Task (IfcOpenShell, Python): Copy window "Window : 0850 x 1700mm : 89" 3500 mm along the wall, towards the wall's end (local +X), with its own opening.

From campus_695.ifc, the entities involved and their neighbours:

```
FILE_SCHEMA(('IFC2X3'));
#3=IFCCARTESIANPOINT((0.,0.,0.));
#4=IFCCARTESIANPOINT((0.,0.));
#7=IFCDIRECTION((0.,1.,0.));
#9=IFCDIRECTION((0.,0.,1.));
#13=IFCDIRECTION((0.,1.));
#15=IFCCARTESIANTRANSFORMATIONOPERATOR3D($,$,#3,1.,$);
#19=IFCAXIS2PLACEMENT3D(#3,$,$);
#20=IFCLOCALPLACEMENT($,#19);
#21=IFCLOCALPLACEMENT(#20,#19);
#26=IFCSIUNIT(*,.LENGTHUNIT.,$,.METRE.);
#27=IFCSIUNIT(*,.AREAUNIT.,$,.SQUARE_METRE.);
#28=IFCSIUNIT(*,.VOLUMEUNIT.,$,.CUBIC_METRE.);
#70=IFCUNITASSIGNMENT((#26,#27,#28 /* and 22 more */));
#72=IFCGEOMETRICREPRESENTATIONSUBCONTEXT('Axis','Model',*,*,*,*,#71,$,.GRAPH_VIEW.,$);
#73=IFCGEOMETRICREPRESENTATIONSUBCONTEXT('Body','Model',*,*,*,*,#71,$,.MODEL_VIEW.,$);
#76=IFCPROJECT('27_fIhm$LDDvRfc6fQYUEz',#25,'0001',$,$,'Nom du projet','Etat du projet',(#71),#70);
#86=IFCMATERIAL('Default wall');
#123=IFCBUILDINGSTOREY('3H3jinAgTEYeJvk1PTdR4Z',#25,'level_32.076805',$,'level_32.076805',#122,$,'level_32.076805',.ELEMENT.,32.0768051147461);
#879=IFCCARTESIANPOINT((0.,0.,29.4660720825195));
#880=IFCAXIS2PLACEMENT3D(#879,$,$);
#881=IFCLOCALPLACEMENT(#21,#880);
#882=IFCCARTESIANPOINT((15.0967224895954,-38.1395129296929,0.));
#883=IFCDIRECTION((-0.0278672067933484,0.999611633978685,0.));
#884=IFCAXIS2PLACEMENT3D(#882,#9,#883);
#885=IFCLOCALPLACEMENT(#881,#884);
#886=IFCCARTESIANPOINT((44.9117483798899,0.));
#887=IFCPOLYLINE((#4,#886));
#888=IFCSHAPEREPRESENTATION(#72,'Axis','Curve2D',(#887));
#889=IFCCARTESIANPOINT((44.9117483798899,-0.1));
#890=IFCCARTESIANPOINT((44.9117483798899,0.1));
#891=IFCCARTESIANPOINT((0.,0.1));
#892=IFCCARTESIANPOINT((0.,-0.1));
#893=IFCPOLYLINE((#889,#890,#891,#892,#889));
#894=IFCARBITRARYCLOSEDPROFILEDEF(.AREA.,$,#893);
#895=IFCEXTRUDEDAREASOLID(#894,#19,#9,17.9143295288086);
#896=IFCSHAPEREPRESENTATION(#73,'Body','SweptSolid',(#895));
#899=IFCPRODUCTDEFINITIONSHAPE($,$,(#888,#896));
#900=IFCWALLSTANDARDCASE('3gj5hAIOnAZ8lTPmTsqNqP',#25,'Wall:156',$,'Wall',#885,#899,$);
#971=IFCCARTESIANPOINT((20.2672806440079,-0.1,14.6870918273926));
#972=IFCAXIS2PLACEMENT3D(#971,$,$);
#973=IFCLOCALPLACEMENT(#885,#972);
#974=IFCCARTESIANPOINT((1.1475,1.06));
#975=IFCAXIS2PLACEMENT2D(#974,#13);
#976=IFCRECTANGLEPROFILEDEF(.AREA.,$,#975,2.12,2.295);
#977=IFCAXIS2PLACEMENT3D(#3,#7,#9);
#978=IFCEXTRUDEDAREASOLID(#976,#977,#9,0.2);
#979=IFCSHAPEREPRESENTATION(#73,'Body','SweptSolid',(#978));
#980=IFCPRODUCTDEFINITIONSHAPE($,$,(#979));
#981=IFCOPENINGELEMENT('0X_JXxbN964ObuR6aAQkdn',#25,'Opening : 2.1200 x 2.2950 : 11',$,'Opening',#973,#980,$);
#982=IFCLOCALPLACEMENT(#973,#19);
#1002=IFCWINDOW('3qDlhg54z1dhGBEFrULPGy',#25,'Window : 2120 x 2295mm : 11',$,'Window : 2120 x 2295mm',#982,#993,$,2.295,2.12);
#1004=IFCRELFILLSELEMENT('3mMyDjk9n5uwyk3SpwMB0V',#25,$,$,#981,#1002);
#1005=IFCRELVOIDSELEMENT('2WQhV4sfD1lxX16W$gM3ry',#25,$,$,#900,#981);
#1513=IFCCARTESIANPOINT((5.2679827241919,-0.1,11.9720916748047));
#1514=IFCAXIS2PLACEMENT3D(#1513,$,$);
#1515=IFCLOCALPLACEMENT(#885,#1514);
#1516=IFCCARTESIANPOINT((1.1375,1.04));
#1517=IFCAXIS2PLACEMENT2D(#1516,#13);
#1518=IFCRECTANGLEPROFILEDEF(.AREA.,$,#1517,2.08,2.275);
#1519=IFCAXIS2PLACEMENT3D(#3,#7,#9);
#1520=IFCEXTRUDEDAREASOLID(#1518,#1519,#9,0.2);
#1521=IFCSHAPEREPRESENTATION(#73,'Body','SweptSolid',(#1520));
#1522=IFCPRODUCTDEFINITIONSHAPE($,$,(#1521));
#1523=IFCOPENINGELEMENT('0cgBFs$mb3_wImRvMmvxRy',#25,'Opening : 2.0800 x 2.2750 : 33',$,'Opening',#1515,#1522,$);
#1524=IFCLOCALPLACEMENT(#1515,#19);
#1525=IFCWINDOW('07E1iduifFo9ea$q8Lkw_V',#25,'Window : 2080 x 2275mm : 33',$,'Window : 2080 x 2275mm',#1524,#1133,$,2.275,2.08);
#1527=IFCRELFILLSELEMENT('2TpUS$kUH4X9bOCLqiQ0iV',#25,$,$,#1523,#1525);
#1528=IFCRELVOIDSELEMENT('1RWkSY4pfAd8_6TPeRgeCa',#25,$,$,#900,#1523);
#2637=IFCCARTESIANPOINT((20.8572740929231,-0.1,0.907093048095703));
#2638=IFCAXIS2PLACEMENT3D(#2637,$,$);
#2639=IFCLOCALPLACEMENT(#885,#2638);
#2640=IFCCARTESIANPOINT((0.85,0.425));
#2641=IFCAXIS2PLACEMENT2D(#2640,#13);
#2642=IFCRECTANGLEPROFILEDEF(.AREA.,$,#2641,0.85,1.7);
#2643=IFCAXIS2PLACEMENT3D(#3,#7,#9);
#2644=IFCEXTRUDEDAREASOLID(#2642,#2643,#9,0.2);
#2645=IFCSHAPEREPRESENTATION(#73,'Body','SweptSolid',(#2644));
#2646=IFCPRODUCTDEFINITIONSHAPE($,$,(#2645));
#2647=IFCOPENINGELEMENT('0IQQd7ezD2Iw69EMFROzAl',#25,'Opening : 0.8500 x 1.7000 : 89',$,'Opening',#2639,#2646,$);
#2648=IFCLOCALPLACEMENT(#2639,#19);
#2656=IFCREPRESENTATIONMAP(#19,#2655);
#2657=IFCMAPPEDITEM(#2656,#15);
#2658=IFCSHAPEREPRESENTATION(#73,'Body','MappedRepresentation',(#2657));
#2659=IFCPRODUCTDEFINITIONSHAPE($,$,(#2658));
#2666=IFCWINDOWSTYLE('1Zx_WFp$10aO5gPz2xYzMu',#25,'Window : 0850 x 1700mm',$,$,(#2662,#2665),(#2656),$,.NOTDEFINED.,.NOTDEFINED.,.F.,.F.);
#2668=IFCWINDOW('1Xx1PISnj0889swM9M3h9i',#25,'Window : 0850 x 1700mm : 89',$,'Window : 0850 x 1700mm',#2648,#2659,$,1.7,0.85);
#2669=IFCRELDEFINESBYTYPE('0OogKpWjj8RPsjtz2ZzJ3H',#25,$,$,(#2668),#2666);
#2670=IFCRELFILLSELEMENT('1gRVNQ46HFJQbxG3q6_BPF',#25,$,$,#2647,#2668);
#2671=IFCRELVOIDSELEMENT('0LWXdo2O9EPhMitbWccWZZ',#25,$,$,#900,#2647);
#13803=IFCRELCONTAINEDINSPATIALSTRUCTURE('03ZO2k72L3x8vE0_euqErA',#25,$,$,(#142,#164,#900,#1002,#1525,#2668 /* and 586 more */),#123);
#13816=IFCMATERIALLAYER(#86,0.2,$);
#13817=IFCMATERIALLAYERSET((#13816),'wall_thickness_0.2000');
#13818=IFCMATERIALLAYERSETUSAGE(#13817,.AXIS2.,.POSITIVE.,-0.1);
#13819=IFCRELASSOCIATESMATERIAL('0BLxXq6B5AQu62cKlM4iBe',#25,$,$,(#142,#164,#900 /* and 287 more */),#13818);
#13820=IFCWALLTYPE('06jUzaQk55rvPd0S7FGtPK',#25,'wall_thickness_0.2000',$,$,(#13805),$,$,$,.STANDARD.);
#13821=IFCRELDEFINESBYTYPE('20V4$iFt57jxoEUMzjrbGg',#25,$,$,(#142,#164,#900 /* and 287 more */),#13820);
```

```python
import ifcopenshell
import ifcopenshell.api.feature
import ifcopenshell.api.geometry
import ifcopenshell.api.root
import ifcopenshell.geom
import ifcopenshell.util.element
import ifcopenshell.util.placement
import ifcopenshell.util.shape
import ifcopenshell.util.unit

model = ifcopenshell.open("campus_695.ifc")
unit_scale = ifcopenshell.util.unit.calculate_unit_scale(model)
settings = ifcopenshell.geom.settings()


def volume(element):
    """Net volume in cubic metres, openings subtracted."""
    shape = ifcopenshell.geom.create_shape(settings, element)
    return ifcopenshell.util.shape.get_volume(shape.geometry)


window = model.by_id(2668)
opening = window.FillsVoids[0].RelatingOpeningElement
wall = opening.VoidsElements[0].RelatingBuildingElement
before = volume(wall)
shift = ifcopenshell.util.placement.get_local_placement(wall.ObjectPlacement)[:3, 0] * 3.5 / unit_scale

# copy_class copies the void relationship, type, container and properties, but no geometry.
new_opening = ifcopenshell.api.root.copy_class(model, product=opening)
new_opening.Representation = ifcopenshell.util.element.copy_deep(
    model, opening.Representation, exclude=["IfcGeometricRepresentationContext", "IfcRepresentationMap"]
)
new_opening.Name = "Opening : 0.8500 x 1.7000"
new_window = ifcopenshell.api.root.copy_class(model, product=window)
new_window.Representation = ifcopenshell.util.element.copy_deep(
    model, window.Representation, exclude=["IfcGeometricRepresentationContext", "IfcRepresentationMap"]
)
new_window.Name = "Window : 0850 x 1700mm"
fills = ifcopenshell.api.feature.add_filling(model, opening=new_opening, element=new_window)
fills.OwnerHistory = new_window.OwnerHistory  # required in IFC2X3

for old, new in ((opening, new_opening), (window, new_window)):
    matrix = ifcopenshell.util.placement.get_local_placement(old.ObjectPlacement)
    matrix[:3, 3] += shift
    ifcopenshell.api.geometry.edit_object_placement(model, product=new, matrix=matrix, is_si=False)

after = volume(wall)

print(f"wall volume {before:.3f} -> {after:.3f} m3")

model.write("campus_695_updated.ifc")
```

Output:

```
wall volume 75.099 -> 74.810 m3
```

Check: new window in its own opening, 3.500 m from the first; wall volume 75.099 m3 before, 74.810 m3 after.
